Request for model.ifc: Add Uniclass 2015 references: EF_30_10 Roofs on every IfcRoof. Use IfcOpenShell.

First a look at what the model holds.

```python
import ifcopenshell

model = ifcopenshell.open("model.ifc")
print(model.schema)
print("classifications:", [c.Name for c in model.by_type("IfcClassification")])
for ifc_class in ("IfcDoor", "IfcRoof", "IfcStair", "IfcWall", "IfcWindow"):
    print(ifc_class, len(model.by_type(ifc_class)))
```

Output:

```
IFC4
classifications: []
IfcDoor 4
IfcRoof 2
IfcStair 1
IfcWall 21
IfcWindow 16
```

```python
import ifcopenshell
import ifcopenshell.api.classification

model = ifcopenshell.open("model.ifc")

system = ifcopenshell.api.classification.add_classification(model, classification="Uniclass 2015")

codes = {
    "IfcRoof": ("EF_30_10", "Roofs"),
}
for ifc_class, (code, name) in codes.items():
    products = model.by_type(ifc_class)
    ifcopenshell.api.classification.add_reference(
        model, products=products, classification=system, identification=code, name=name
    )
    print(code, len(products))

model.write("model-out.ifc")
```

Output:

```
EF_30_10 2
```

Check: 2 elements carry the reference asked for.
